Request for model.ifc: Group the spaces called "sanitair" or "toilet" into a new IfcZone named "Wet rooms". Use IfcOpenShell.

First a look at what the model holds.

```python
import ifcopenshell

model = ifcopenshell.open("model.ifc")
print(model.schema)
seen = {}
for space in model.by_type("IfcSpace"):
    seen[space.LongName] = seen.get(space.LongName, 0) + 1
for name, count in sorted(seen.items(), key=str):
    print(count, "x", name)
print("zones:", [z.Name for z in model.by_type("IfcZone")][:20])
```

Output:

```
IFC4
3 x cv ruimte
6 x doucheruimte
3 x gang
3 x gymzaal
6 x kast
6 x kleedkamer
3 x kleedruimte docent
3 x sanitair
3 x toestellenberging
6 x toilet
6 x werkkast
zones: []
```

```python
import ifcopenshell
import ifcopenshell.api.group
import ifcopenshell.api.root

model = ifcopenshell.open("model.ifc")

names = {"sanitair", "toilet"}
spaces = [s for s in model.by_type("IfcSpace") if s.LongName in names]

zone = ifcopenshell.api.root.create_entity(model, ifc_class="IfcZone", name="Wet rooms")
ifcopenshell.api.group.assign_group(model, products=spaces, group=zone)
print(len(spaces), "spaces in", zone.Name)

model.write("model_edited.ifc")
```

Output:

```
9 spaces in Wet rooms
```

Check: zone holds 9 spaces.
